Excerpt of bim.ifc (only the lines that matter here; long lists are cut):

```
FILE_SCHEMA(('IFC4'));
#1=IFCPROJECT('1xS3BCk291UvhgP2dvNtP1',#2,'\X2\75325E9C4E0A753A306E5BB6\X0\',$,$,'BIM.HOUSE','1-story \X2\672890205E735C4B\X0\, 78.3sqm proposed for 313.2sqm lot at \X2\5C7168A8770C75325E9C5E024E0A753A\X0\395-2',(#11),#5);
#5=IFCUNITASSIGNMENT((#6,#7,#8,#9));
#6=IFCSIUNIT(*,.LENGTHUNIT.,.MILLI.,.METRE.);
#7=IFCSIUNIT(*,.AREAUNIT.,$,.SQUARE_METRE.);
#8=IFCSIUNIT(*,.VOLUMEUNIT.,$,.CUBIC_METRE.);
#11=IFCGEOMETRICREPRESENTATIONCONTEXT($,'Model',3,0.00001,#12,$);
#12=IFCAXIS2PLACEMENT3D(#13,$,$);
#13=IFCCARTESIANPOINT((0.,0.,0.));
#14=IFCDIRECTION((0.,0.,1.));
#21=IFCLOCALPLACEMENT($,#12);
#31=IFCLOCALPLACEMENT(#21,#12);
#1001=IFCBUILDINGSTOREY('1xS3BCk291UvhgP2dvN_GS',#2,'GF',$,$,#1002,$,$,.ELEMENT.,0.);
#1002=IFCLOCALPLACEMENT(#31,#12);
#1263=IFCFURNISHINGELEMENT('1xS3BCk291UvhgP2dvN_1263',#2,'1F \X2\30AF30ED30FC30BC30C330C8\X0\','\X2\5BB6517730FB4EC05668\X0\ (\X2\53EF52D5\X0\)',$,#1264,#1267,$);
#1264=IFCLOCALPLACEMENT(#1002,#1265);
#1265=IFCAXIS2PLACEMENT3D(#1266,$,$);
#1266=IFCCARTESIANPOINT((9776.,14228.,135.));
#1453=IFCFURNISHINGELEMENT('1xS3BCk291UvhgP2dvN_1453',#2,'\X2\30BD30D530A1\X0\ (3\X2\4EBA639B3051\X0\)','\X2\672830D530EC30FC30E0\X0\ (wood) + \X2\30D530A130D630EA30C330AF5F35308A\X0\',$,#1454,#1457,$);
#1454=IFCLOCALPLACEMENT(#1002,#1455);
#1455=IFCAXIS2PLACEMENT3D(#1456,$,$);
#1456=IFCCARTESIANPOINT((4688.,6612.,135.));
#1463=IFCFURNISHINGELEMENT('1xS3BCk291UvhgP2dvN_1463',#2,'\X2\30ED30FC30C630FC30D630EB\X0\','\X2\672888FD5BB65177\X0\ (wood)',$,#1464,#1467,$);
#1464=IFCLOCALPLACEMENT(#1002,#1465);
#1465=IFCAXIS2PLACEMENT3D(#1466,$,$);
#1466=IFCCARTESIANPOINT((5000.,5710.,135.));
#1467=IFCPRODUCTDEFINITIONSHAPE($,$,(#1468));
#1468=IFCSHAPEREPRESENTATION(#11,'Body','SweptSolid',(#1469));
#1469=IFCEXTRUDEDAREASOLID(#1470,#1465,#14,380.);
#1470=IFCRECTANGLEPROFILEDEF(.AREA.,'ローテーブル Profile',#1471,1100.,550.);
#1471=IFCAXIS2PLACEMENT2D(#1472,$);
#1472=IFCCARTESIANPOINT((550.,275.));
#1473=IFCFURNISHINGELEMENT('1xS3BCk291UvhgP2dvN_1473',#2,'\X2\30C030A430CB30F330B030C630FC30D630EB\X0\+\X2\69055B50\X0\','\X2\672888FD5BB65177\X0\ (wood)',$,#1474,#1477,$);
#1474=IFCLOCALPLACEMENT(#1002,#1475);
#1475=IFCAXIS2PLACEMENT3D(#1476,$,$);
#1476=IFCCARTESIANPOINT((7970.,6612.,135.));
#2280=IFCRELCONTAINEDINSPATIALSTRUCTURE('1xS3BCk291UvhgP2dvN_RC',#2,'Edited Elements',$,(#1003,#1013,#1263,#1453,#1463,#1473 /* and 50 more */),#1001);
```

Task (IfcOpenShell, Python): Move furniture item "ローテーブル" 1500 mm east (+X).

```python
import ifcopenshell
import ifcopenshell.api.geometry
import ifcopenshell.util.placement
import ifcopenshell.util.unit

model = ifcopenshell.open("bim.ifc")
unit_scale = ifcopenshell.util.unit.calculate_unit_scale(model)

item = model.by_guid("1xS3BCk291UvhgP2dvN_1463")
matrix = ifcopenshell.util.placement.get_local_placement(item.ObjectPlacement)
matrix[0, 3] += 1.5 / unit_scale
ifcopenshell.api.geometry.edit_object_placement(model, product=item, matrix=matrix, is_si=False)

print(ifcopenshell.util.placement.get_local_placement(item.ObjectPlacement).round(3) + 0.0)

model.write("bim_rev.ifc")
```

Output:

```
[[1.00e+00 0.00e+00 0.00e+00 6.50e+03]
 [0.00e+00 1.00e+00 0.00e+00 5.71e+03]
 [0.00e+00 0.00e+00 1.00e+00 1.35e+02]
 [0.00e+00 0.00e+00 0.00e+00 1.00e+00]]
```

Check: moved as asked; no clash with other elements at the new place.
